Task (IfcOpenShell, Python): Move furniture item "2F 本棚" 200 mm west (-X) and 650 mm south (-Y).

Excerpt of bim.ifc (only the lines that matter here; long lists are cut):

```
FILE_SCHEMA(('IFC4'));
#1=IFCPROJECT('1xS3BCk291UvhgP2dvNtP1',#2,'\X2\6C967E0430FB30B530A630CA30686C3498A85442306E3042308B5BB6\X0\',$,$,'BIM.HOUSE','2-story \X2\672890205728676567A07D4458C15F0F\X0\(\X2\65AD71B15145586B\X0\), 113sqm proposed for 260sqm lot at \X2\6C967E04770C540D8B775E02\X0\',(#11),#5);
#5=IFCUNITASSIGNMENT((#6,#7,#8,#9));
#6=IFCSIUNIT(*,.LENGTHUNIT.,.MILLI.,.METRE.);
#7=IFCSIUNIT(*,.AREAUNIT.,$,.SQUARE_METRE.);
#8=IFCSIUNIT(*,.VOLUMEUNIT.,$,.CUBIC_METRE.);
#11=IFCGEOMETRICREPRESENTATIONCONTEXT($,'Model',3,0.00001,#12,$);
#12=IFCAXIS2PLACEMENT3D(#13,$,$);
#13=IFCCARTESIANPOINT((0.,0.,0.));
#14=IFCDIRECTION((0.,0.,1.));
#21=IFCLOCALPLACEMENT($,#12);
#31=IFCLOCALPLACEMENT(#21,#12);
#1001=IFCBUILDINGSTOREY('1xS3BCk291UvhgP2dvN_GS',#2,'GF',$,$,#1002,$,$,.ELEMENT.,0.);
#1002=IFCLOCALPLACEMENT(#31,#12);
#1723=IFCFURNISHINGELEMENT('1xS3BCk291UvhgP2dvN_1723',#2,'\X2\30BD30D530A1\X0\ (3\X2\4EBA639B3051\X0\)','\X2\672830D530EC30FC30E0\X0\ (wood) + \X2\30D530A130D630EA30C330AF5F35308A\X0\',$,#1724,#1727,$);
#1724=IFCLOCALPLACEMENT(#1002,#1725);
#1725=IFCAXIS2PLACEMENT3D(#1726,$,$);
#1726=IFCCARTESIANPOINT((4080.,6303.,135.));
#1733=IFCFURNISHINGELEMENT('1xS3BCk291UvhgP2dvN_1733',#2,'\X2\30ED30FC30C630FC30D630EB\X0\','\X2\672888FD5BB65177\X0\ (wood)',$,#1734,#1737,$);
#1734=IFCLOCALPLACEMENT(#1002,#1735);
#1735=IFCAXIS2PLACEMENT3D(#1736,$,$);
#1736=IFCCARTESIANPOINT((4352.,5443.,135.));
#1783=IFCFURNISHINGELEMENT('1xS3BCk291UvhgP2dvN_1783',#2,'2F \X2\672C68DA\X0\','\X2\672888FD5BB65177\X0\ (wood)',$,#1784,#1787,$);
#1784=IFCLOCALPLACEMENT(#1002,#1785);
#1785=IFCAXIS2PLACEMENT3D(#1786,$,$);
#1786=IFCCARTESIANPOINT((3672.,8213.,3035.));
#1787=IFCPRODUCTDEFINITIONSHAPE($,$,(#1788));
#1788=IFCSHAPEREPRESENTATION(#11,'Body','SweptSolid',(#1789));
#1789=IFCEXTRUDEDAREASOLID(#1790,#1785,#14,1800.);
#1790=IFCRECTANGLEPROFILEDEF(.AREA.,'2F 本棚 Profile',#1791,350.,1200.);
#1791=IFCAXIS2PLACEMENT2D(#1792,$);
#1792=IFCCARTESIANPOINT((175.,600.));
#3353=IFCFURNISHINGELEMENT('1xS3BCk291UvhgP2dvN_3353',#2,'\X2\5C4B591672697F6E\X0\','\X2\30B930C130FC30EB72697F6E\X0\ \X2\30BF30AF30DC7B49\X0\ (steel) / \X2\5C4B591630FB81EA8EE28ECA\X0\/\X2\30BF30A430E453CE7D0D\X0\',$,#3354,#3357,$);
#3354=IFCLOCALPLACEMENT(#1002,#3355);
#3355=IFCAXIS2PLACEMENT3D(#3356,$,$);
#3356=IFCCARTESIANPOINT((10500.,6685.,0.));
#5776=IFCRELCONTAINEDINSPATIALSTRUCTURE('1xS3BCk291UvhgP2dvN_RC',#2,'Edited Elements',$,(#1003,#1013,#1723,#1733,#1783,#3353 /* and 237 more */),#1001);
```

```python
import ifcopenshell
import ifcopenshell.api.geometry
import ifcopenshell.util.placement

model = ifcopenshell.open("bim.ifc")

item = model.by_guid("1xS3BCk291UvhgP2dvN_1783")
matrix = ifcopenshell.util.placement.get_local_placement(item.ObjectPlacement)
matrix[0, 3] -= 200.0
matrix[1, 3] -= 650.0
ifcopenshell.api.geometry.edit_object_placement(model, product=item, matrix=matrix, is_si=False)

print(ifcopenshell.util.placement.get_local_placement(item.ObjectPlacement).round(3) + 0.0)

model.write("bim-out.ifc")
```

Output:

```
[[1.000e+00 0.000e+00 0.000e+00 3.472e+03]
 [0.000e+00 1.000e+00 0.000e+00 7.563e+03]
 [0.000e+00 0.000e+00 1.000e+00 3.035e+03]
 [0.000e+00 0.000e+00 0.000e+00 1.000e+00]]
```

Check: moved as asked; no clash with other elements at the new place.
